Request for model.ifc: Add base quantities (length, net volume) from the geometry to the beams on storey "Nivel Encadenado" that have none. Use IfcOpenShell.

First a look at what the model holds.

```python
import ifcopenshell
import ifcopenshell.util.element
import ifcopenshell.util.unit

model = ifcopenshell.open("model.ifc")
print(model.schema)
for unit_type in ("LENGTHUNIT", "AREAUNIT", "VOLUMEUNIT"):
    print(unit_type, ifcopenshell.util.unit.calculate_unit_scale(model, unit_type))
storey = next(s for s in model.by_type("IfcBuildingStorey") if s.Name == "Nivel Encadenado")
beams = [e for e in ifcopenshell.util.element.get_decomposition(storey) if e.is_a("IfcBeam")]
for e in sorted(beams, key=lambda e: e.id()):
    print(e.id(), e.is_a(), e.Name, list(ifcopenshell.util.element.get_psets(e, qtos_only=True)), sep=" | ")
```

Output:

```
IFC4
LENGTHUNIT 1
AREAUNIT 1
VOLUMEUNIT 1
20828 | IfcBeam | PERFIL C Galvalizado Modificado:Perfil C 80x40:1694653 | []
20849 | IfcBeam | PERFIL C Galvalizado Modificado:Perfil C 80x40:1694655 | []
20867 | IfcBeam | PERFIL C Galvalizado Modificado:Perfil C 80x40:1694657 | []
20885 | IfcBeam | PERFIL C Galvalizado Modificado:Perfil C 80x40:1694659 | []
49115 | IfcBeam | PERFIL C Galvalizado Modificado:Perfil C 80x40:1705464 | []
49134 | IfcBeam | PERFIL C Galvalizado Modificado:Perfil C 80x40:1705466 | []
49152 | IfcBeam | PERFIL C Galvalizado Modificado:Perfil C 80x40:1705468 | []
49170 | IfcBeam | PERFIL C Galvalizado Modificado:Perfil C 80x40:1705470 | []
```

```python
import ifcopenshell
import ifcopenshell.api.pset
import ifcopenshell.geom
import ifcopenshell.util.element
import ifcopenshell.util.shape
import ifcopenshell.util.unit

model = ifcopenshell.open("model.ifc")
unit_scale = ifcopenshell.util.unit.calculate_unit_scale(model)
volume_scale = ifcopenshell.util.unit.calculate_unit_scale(model, "VOLUMEUNIT")
settings = ifcopenshell.geom.settings()

storey = next(s for s in model.by_type("IfcBuildingStorey") if s.Name == "Nivel Encadenado")
beams = [e for e in ifcopenshell.util.element.get_decomposition(storey) if e.is_a("IfcBeam")]

for e in sorted(beams, key=lambda e: e.id()):
    if ifcopenshell.util.element.get_psets(e, qtos_only=True, should_inherit=False):
        continue
    # Geometry comes back in metres, in the element's own axes.
    shape = ifcopenshell.geom.create_shape(settings, e)
    values = {
        "Length": ifcopenshell.util.shape.get_max_xyz(shape.geometry) / unit_scale,
        "NetVolume": ifcopenshell.util.shape.get_volume(shape.geometry) / volume_scale,
    }
    qto = ifcopenshell.api.pset.add_qto(model, product=e, name="Qto_BeamBaseQuantities")
    ifcopenshell.api.pset.edit_qto(model, qto=qto, properties=values)
    print(e.id(), {k: round(v, 3) for k, v in values.items()})

model.write("model_edited.ifc")
```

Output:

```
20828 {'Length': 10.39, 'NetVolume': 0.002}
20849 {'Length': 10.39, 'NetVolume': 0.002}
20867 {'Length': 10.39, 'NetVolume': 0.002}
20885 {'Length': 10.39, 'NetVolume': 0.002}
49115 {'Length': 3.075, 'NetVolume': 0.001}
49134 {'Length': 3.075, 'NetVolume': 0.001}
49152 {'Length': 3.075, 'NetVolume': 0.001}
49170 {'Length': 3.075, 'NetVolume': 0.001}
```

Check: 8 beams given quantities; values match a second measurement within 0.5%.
